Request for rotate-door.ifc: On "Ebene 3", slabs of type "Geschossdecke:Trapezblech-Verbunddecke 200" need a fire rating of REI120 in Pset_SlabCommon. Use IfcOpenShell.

First a look at what the model holds.

```python
import ifcopenshell
import ifcopenshell.util.element

model = ifcopenshell.open("rotate-door.ifc")
print(model.schema)
storey = next(s for s in model.by_type("IfcBuildingStorey") if s.Name == "Ebene 3")
slabs = [e for e in ifcopenshell.util.element.get_decomposition(storey) if e.is_a("IfcSlab")]
seen = {}
for e in slabs:
    element_type = ifcopenshell.util.element.get_type(e)
    key = (element_type.Name if element_type != e and element_type else None, ifcopenshell.util.element.get_pset(e, "Pset_SlabCommon", "FireRating"))
    seen[key] = seen.get(key, 0) + 1
for (name, value), count in sorted(seen.items(), key=str):
    print(count, "x", name, "|", value)
```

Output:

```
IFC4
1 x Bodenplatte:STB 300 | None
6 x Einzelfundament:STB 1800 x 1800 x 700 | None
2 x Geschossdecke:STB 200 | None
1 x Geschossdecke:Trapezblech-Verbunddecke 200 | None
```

```python
import ifcopenshell
import ifcopenshell.api.pset
import ifcopenshell.util.element

model = ifcopenshell.open("rotate-door.ifc")

storey = next(s for s in model.by_type("IfcBuildingStorey") if s.Name == "Ebene 3")
slabs = [e for e in ifcopenshell.util.element.get_decomposition(storey) if e.is_a("IfcSlab")]

count = 0
for e in slabs:
    element_type = ifcopenshell.util.element.get_type(e)
    if element_type in (None, e) or element_type.Name != "Geschossdecke:Trapezblech-Verbunddecke 200":
        continue
    # add_pset returns the element's existing set when there is one.
    pset = ifcopenshell.api.pset.add_pset(model, product=e, name="Pset_SlabCommon")
    ifcopenshell.api.pset.edit_pset(model, pset=pset, properties={"FireRating": "REI120"})
    count += 1

print(count, "slabs updated")

model.write("rotate-door-out.ifc")
```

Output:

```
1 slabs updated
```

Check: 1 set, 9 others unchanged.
